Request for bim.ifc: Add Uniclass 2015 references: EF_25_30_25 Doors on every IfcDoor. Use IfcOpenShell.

First a look at what the model holds.

```python
import ifcopenshell

model = ifcopenshell.open("bim.ifc")
print(model.schema)
print("classifications:", [c.Name for c in model.by_type("IfcClassification")])
for ifc_class in ("IfcDoor", "IfcRoof", "IfcStair", "IfcWall", "IfcWindow"):
    print(ifc_class, len(model.by_type(ifc_class)))
```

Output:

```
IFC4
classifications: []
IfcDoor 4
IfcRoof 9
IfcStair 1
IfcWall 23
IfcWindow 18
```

```python
import ifcopenshell
import ifcopenshell.api.classification

model = ifcopenshell.open("bim.ifc")

system = ifcopenshell.api.classification.add_classification(model, classification="Uniclass 2015")

codes = {
    "IfcDoor": ("EF_25_30_25", "Doors"),
}
for ifc_class, (code, name) in codes.items():
    products = model.by_type(ifc_class)
    ifcopenshell.api.classification.add_reference(
        model, products=products, classification=system, identification=code, name=name
    )
    print(code, len(products))

model.write("bim_edited.ifc")
```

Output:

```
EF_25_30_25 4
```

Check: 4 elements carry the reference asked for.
